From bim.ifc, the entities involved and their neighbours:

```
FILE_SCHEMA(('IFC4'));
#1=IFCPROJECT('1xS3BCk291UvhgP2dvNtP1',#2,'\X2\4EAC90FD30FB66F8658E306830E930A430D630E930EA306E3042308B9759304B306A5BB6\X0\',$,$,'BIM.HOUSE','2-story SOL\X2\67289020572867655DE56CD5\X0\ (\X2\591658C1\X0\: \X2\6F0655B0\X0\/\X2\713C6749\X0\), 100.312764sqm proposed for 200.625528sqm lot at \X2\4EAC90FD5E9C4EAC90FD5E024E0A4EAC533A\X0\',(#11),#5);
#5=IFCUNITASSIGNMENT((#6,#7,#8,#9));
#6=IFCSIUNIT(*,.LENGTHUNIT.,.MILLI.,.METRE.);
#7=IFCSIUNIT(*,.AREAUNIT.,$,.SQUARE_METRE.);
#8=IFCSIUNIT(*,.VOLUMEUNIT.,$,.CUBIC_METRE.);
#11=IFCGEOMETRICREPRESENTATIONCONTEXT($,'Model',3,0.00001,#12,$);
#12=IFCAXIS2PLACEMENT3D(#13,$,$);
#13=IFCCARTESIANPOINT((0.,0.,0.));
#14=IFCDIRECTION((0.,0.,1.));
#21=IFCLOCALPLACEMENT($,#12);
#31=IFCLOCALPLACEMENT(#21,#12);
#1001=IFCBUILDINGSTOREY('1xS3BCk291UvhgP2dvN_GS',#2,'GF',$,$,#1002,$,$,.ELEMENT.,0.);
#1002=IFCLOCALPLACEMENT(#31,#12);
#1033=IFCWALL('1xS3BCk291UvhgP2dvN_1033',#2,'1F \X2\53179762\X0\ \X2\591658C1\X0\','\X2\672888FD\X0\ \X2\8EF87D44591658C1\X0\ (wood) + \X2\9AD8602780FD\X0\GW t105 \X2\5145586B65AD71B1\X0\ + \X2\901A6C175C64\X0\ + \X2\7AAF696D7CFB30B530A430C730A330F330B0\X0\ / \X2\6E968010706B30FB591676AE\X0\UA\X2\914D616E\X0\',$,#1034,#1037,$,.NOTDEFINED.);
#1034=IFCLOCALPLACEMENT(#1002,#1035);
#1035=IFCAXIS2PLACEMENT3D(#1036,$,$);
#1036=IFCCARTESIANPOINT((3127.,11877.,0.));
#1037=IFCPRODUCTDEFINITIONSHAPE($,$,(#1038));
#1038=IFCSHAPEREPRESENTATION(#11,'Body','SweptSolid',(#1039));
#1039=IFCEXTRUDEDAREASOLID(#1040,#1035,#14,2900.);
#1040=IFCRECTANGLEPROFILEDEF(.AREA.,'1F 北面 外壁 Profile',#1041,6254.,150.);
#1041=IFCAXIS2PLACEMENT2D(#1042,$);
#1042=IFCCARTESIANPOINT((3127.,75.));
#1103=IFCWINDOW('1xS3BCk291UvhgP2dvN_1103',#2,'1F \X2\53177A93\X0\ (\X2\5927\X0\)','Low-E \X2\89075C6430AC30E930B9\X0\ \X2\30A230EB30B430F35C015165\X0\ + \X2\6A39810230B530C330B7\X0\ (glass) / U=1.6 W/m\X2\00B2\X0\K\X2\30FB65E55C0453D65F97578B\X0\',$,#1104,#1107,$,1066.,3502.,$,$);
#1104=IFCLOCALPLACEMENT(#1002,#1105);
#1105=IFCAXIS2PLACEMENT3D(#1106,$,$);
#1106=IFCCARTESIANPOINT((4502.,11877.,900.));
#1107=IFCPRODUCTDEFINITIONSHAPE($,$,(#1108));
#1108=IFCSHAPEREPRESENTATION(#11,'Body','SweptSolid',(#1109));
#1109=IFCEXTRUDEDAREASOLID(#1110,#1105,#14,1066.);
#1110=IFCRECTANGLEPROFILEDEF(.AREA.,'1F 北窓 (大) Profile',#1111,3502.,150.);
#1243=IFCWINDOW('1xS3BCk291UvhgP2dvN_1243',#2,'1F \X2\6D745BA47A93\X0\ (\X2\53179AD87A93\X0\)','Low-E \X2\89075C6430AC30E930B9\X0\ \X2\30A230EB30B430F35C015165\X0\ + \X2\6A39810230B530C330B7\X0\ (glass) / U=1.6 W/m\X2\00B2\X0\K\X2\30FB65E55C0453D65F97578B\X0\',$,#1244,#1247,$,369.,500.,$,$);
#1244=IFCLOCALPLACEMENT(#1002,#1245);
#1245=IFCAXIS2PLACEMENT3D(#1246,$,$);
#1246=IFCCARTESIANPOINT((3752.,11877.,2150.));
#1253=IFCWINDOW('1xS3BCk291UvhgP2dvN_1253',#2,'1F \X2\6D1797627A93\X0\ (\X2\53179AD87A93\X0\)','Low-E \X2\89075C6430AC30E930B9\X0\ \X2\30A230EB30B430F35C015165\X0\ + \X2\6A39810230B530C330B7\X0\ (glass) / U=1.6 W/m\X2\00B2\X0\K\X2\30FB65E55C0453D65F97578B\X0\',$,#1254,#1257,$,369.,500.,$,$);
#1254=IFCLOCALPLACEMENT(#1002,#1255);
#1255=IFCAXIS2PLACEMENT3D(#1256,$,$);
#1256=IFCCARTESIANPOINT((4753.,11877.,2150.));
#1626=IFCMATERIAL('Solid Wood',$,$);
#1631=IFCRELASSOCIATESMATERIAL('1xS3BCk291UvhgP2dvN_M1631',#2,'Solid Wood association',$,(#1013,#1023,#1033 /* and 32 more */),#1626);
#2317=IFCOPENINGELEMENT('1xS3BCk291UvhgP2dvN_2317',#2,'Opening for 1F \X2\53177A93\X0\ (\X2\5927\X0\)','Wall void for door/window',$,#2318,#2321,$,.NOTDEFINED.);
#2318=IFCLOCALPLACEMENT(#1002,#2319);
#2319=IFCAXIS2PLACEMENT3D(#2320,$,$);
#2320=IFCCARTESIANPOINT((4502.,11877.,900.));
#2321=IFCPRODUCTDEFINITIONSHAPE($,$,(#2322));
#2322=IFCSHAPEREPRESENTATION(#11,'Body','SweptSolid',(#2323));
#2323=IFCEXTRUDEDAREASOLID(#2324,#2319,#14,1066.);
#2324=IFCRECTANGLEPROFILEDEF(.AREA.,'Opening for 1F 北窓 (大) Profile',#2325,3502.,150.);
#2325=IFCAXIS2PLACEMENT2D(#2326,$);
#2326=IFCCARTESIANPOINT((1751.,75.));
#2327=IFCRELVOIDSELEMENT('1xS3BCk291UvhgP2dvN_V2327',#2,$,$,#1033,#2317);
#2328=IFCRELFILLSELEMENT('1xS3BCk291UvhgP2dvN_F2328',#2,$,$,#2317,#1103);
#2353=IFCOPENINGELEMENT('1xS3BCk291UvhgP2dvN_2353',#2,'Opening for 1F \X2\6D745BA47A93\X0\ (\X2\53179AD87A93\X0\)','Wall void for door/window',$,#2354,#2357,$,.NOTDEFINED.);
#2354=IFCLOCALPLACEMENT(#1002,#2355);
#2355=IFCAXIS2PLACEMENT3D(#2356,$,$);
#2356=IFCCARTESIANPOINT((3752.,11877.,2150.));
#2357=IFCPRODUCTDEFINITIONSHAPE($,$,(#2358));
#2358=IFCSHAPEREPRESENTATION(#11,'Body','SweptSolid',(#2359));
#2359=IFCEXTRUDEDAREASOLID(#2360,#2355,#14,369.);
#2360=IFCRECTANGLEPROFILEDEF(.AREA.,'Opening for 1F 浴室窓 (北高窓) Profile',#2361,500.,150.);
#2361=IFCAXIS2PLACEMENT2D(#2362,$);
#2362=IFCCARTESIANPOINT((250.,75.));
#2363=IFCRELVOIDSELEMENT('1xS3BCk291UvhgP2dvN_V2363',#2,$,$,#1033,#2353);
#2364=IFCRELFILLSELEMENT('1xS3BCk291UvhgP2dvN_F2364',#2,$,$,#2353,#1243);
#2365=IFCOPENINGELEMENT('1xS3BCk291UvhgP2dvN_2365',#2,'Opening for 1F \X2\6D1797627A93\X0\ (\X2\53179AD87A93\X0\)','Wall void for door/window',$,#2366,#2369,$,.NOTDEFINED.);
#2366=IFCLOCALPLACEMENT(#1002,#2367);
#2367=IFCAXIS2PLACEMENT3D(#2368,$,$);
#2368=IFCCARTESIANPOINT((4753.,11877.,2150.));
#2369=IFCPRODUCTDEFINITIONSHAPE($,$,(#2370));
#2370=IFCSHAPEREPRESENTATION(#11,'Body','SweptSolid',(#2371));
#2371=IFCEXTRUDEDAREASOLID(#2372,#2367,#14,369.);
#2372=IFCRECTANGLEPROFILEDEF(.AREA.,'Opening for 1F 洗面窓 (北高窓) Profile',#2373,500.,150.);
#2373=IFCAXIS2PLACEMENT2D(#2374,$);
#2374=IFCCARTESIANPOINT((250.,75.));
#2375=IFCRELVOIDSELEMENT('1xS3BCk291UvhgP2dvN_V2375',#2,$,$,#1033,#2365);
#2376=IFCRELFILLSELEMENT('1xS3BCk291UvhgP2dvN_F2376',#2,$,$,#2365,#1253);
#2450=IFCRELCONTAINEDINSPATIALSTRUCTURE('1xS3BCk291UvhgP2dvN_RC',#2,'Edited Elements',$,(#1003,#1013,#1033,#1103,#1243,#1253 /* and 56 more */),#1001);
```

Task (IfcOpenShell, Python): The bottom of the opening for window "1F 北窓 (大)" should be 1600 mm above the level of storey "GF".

```python
import numpy as np
import ifcopenshell
import ifcopenshell.api.geometry
import ifcopenshell.geom
import ifcopenshell.util.element
import ifcopenshell.util.placement
import ifcopenshell.util.shape
import ifcopenshell.util.unit

model = ifcopenshell.open("bim.ifc")
unit_scale = ifcopenshell.util.unit.calculate_unit_scale(model)

window = model.by_id(1103)
opening = window.FillsVoids[0].RelatingOpeningElement
storey = ifcopenshell.util.element.get_container(window, ifc_class="IfcBuildingStorey")
level = ifcopenshell.util.placement.get_local_placement(storey.ObjectPlacement)[2, 3]

# The opening's origin need not be at the sill, so measure its lowest point.
shape = ifcopenshell.geom.create_shape(ifcopenshell.geom.settings(), opening)
bottom = ifcopenshell.util.shape.get_shape_bottom_elevation(shape, shape.geometry) / unit_scale
dz = level + 1.6 / unit_scale - bottom

shift = np.array([0.0, 0.0, dz])
# The window is not placed relative to its opening, so move both.
for product in (opening, window):
    matrix = ifcopenshell.util.placement.get_local_placement(product.ObjectPlacement)
    matrix[:3, 3] += shift
    ifcopenshell.api.geometry.edit_object_placement(model, product=product, matrix=matrix, is_si=False)

print(f"moved by {dz * unit_scale:+.3f} m")

model.write("bim_rev.ifc")
```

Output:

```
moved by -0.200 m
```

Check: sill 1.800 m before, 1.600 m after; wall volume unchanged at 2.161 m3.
